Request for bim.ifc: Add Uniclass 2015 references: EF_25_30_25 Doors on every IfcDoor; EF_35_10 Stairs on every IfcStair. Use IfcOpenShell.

First a look at what the model holds.

```python
import ifcopenshell

model = ifcopenshell.open("bim.ifc")
print(model.schema)
print("classifications:", [c.Name for c in model.by_type("IfcClassification")])
for ifc_class in ("IfcDoor", "IfcRoof", "IfcStair", "IfcWall", "IfcWindow"):
    print(ifc_class, len(model.by_type(ifc_class)))
```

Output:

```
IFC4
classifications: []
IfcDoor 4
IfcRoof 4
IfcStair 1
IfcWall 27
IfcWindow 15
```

```python
import ifcopenshell
import ifcopenshell.api.classification

model = ifcopenshell.open("bim.ifc")

system = ifcopenshell.api.classification.add_classification(model, classification="Uniclass 2015")

codes = {
    "IfcDoor": ("EF_25_30_25", "Doors"),
    "IfcStair": ("EF_35_10", "Stairs"),
}
for ifc_class, (code, name) in codes.items():
    products = model.by_type(ifc_class)
    ifcopenshell.api.classification.add_reference(
        model, products=products, classification=system, identification=code, name=name
    )
    print(code, len(products))

model.write("bim_rev.ifc")
```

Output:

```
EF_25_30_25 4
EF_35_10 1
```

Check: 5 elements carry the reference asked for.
